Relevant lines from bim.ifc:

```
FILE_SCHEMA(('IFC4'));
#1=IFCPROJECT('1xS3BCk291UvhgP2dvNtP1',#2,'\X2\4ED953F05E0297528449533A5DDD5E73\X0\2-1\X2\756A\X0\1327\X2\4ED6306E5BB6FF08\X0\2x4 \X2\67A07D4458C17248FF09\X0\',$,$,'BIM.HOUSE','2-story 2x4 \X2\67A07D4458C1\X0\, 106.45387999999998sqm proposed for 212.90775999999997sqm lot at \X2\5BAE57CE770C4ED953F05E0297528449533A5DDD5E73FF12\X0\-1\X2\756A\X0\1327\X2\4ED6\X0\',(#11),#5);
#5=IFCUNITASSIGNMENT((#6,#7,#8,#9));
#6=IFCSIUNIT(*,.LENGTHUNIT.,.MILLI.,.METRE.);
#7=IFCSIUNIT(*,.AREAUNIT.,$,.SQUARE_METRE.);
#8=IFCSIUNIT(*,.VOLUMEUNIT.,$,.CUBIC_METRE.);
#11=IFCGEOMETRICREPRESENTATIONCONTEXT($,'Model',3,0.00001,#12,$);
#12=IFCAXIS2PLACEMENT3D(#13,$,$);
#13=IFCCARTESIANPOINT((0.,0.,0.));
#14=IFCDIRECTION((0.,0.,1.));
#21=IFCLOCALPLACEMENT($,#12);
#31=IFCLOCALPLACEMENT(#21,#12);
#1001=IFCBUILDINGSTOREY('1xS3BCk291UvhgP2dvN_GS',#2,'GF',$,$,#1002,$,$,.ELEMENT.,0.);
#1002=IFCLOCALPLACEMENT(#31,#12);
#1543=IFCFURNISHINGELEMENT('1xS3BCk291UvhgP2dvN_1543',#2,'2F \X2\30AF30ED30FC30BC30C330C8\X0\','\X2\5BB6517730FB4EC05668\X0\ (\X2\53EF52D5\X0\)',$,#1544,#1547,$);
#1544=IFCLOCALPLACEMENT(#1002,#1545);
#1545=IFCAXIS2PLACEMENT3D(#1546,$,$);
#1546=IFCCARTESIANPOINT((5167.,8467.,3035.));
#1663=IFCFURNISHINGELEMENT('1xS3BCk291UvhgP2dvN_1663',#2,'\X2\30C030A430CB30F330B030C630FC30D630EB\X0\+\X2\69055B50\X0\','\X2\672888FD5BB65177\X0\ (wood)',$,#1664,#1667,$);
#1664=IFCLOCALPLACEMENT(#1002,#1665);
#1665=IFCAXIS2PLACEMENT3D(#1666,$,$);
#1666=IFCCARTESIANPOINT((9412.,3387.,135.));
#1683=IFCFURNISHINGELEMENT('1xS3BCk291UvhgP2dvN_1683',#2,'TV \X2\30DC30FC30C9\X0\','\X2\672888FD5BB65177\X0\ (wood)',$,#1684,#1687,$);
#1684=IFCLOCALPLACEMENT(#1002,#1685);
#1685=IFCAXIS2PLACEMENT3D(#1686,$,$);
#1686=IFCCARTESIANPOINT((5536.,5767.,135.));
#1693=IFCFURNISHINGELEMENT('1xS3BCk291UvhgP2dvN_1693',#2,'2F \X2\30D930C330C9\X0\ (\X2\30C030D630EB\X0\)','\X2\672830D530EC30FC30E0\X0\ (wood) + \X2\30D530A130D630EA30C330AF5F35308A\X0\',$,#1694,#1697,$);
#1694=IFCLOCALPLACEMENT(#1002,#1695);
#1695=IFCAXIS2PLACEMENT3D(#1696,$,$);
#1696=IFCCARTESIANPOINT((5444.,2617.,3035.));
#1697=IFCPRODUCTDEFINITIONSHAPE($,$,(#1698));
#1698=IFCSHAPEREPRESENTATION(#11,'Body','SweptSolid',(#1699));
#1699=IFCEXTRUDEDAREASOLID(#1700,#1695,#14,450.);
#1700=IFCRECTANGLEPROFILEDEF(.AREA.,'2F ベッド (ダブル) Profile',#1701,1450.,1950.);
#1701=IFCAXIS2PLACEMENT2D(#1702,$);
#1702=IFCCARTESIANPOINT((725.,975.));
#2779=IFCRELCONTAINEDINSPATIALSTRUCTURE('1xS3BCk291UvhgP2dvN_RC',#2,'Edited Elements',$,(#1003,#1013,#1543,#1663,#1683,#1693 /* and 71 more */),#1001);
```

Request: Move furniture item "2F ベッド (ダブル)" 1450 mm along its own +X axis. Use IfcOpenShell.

```python
import ifcopenshell
import ifcopenshell.api.geometry
import ifcopenshell.util.placement

model = ifcopenshell.open("bim.ifc")

item = model.by_guid("1xS3BCk291UvhgP2dvN_1693")
matrix = ifcopenshell.util.placement.get_local_placement(item.ObjectPlacement)
matrix[:3, 3] += matrix[:3, 0] * 1450.0
ifcopenshell.api.geometry.edit_object_placement(model, product=item, matrix=matrix, is_si=False)

print(ifcopenshell.util.placement.get_local_placement(item.ObjectPlacement).round(3) + 0.0)

model.write("bim-out.ifc")
```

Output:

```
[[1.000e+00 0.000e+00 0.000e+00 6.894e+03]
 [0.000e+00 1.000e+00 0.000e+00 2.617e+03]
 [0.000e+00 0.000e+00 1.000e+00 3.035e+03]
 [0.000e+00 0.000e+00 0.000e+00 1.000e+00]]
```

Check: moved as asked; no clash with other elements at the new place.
